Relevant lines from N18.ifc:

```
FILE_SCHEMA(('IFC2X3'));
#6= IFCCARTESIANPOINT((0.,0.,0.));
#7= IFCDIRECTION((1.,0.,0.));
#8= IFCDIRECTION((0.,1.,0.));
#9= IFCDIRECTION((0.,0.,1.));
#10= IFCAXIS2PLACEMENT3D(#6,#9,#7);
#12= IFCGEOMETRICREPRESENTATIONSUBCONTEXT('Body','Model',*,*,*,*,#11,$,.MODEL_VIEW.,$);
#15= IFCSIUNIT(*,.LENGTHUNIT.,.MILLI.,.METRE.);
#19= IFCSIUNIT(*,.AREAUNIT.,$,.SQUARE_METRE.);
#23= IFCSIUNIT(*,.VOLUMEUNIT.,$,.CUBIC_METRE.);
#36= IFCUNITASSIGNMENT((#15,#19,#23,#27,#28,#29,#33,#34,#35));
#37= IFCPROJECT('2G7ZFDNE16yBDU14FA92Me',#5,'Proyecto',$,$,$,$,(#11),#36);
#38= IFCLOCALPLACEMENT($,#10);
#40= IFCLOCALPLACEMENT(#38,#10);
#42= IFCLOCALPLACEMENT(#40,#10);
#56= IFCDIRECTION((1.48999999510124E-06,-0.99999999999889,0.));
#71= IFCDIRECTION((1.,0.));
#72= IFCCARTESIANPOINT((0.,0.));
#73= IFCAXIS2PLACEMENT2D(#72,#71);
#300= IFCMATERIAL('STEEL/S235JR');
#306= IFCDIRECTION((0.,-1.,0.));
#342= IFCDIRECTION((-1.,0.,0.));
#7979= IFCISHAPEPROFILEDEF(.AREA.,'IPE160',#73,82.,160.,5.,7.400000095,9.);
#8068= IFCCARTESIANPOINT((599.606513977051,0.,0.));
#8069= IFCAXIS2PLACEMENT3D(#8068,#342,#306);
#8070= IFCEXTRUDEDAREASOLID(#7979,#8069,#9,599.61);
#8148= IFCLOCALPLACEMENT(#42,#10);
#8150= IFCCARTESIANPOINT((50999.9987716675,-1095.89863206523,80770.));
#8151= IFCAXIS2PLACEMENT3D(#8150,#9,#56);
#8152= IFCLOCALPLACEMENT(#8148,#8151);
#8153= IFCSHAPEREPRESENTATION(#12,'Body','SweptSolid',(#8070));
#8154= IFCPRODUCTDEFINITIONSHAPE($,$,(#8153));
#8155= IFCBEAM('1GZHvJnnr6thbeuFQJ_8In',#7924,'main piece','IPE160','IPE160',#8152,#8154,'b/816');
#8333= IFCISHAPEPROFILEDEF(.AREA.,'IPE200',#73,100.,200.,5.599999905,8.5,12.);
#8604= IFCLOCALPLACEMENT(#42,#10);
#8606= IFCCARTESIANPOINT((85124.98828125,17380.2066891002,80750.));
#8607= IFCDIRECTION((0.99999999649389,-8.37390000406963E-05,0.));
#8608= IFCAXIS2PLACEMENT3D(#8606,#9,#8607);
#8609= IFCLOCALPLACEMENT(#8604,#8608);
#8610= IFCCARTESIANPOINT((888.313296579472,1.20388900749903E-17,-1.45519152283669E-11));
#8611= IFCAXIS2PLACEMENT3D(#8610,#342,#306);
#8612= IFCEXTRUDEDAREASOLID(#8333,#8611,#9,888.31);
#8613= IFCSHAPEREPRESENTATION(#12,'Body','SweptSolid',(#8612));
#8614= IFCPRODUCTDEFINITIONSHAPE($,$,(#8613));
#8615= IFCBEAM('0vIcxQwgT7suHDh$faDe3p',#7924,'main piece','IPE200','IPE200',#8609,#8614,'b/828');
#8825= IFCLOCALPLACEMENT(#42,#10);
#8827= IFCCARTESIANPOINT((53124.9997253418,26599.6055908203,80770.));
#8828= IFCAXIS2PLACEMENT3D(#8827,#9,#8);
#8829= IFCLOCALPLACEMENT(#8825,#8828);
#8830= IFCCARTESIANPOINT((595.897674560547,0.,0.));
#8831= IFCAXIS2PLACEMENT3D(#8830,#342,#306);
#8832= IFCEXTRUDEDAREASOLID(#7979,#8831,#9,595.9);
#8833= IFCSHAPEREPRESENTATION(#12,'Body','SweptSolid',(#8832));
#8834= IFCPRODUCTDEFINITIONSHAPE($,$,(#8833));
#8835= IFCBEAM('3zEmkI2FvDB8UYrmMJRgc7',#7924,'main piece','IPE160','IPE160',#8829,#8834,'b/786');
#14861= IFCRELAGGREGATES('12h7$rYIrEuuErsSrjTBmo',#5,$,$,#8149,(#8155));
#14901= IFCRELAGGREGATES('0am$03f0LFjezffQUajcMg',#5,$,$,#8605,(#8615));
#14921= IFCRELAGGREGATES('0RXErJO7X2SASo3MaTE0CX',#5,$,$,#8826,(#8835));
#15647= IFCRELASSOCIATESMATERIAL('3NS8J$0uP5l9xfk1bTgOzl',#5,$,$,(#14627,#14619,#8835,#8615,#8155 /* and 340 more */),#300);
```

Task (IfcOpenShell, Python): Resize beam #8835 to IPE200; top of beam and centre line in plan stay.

```python
import ifcopenshell
import ifcopenshell.util.element
import ifcopenshell.util.representation

model = ifcopenshell.open("N18.ifc")

member = model.by_id(8835)
source = next(p for p in model.by_type("IfcIShapeProfileDef") if p.ProfileName == "IPE200")

body = ifcopenshell.util.representation.get_representation(member, "Model", "Body")
solid = body.Items[0]
old_profile = solid.SweptArea

# Copy the section's sizes but keep this member's own profile position.
profile = ifcopenshell.util.element.copy(model, source)
# Profiles are centred, so shift by half the change in depth to hold the top.
shift = (old_profile.OverallDepth - profile.OverallDepth) / 2
x, y = old_profile.Position.Location.Coordinates
up = (0.0, 1.0)  # upwards, in the solid's own plane
location = model.createIfcCartesianPoint((x + up[0] * shift, y + up[1] * shift))
profile.Position = model.createIfcAxis2Placement2D(location, old_profile.Position.RefDirection)
solid.SweptArea = profile
if not model.get_total_inverses(old_profile):
    ifcopenshell.util.element.remove_deep2(model, old_profile)
member.Description = member.Description.replace("IPE160", "IPE200")
member.ObjectType = member.ObjectType.replace("IPE160", "IPE200")

print(solid.SweptArea)

model.write("N18_updated.ifc")
```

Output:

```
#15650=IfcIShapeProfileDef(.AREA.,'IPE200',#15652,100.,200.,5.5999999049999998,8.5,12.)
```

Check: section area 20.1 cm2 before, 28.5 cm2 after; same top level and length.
